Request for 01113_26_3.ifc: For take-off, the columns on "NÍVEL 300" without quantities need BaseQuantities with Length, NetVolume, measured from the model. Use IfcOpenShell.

First a look at what the model holds.

```python
import ifcopenshell
import ifcopenshell.util.element
import ifcopenshell.util.unit

model = ifcopenshell.open("01113_26_3.ifc")
print(model.schema)
for unit_type in ("LENGTHUNIT", "AREAUNIT", "VOLUMEUNIT"):
    print(unit_type, ifcopenshell.util.unit.calculate_unit_scale(model, unit_type))
storey = next(s for s in model.by_type("IfcBuildingStorey") if s.Name == "NÍVEL 300")
columns = [e for e in ifcopenshell.util.element.get_decomposition(storey) if e.is_a("IfcColumn")]
for e in sorted(columns, key=lambda e: e.id()):
    print(e.id(), e.is_a(), e.Name, list(ifcopenshell.util.element.get_psets(e, qtos_only=True)), sep=" | ")
```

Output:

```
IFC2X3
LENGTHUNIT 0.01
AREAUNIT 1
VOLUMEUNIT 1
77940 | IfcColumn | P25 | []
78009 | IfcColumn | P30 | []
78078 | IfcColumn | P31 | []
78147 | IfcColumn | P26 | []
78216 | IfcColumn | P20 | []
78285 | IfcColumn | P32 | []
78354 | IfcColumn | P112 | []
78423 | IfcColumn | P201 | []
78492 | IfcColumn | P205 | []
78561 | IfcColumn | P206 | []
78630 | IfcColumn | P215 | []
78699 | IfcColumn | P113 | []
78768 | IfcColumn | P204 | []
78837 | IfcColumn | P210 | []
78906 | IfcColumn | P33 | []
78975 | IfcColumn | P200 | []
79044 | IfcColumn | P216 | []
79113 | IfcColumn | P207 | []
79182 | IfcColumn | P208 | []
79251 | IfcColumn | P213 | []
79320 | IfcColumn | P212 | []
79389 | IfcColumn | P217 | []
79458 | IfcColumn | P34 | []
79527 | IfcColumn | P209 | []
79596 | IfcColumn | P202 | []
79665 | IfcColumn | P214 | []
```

```python
import ifcopenshell
import ifcopenshell.api.pset
import ifcopenshell.geom
import ifcopenshell.util.element
import ifcopenshell.util.shape
import ifcopenshell.util.unit

model = ifcopenshell.open("01113_26_3.ifc")
unit_scale = ifcopenshell.util.unit.calculate_unit_scale(model)
volume_scale = ifcopenshell.util.unit.calculate_unit_scale(model, "VOLUMEUNIT")
settings = ifcopenshell.geom.settings()

storey = next(s for s in model.by_type("IfcBuildingStorey") if s.Name == "NÍVEL 300")
columns = [e for e in ifcopenshell.util.element.get_decomposition(storey) if e.is_a("IfcColumn")]

for e in sorted(columns, key=lambda e: e.id()):
    if ifcopenshell.util.element.get_psets(e, qtos_only=True, should_inherit=False):
        continue
    # Geometry comes back in metres, in the element's own axes.
    shape = ifcopenshell.geom.create_shape(settings, e)
    values = {
        "Length": ifcopenshell.util.shape.get_z(shape.geometry) / unit_scale,
        "NetVolume": ifcopenshell.util.shape.get_volume(shape.geometry) / volume_scale,
    }
    qto = ifcopenshell.api.pset.add_qto(model, product=e, name="BaseQuantities")
    ifcopenshell.api.pset.edit_qto(model, qto=qto, properties=values)
    print(e.id(), {k: round(v, 3) for k, v in values.items()})

model.write("01113_26_3_updated.ifc")
```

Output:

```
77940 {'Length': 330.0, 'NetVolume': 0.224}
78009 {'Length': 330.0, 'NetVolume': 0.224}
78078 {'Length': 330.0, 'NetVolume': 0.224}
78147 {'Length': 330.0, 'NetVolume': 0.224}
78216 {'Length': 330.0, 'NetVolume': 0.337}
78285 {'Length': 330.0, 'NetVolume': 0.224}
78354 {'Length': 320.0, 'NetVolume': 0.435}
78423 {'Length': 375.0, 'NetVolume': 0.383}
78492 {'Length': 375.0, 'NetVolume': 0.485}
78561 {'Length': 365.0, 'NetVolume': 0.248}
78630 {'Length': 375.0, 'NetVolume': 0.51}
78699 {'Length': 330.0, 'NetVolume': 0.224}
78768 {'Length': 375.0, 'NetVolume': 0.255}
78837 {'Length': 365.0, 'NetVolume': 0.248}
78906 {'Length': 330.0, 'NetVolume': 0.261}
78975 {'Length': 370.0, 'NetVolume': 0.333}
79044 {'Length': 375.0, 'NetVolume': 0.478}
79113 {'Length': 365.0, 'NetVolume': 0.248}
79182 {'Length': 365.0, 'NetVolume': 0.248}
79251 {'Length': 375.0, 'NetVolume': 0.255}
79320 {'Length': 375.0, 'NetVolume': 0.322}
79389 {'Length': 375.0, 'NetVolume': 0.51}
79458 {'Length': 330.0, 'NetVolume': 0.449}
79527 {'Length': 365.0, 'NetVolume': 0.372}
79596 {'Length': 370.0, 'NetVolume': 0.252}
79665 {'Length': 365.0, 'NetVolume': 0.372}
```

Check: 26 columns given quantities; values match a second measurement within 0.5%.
